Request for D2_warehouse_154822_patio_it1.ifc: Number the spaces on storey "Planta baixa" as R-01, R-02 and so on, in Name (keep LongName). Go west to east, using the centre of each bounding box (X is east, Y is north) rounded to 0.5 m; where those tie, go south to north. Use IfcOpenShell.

First a look at what the model holds.

```python
import ifcopenshell
import ifcopenshell.util.element
import ifcopenshell.util.placement

model = ifcopenshell.open("D2_warehouse_154822_patio_it1.ifc")
print(model.schema)
storey = next(s for s in model.by_type("IfcBuildingStorey") if s.Name == "Planta baixa")
spaces = [e for e in ifcopenshell.util.element.get_decomposition(storey) if e.is_a("IfcSpace")]
for e in sorted(spaces, key=lambda e: e.id()):
    origin = ifcopenshell.util.placement.get_local_placement(e.ObjectPlacement)[:3, 3]
    print(e.id(), e.Name, e.LongName, origin.round(2) + 0.0, sep=" | ")
```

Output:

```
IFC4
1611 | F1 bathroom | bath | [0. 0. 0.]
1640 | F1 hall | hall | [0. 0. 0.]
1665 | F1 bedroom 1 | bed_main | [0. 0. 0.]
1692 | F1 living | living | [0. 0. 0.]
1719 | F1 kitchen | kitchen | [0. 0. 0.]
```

```python
import ifcopenshell
import ifcopenshell.geom
import ifcopenshell.util.element
import ifcopenshell.util.shape

model = ifcopenshell.open("D2_warehouse_154822_patio_it1.ifc")
settings = ifcopenshell.geom.settings()
settings.set("use-world-coords", True)


def centre(element):
    shape = ifcopenshell.geom.create_shape(settings, element)
    return ifcopenshell.util.shape.get_bbox_centroid(shape.geometry)


storey = next(s for s in model.by_type("IfcBuildingStorey") if s.Name == "Planta baixa")
spaces = [e for e in ifcopenshell.util.element.get_decomposition(storey) if e.is_a("IfcSpace")]

# Insertion points can sit at a corner or the storey origin, so sort by the geometry (in metres).
centres = {e: centre(e) for e in spaces}
spaces.sort(key=lambda e: (round(centres[e][0] / 0.5), centres[e][1]))

for i, e in enumerate(spaces, start=1):
    number = f"R-{i:02d}"
    e.Name = number
    print(e.id(), number)

model.write("D2_warehouse_154822_patio_it1_updated.ifc")
```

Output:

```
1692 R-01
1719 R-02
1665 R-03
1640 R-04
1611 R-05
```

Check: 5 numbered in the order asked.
